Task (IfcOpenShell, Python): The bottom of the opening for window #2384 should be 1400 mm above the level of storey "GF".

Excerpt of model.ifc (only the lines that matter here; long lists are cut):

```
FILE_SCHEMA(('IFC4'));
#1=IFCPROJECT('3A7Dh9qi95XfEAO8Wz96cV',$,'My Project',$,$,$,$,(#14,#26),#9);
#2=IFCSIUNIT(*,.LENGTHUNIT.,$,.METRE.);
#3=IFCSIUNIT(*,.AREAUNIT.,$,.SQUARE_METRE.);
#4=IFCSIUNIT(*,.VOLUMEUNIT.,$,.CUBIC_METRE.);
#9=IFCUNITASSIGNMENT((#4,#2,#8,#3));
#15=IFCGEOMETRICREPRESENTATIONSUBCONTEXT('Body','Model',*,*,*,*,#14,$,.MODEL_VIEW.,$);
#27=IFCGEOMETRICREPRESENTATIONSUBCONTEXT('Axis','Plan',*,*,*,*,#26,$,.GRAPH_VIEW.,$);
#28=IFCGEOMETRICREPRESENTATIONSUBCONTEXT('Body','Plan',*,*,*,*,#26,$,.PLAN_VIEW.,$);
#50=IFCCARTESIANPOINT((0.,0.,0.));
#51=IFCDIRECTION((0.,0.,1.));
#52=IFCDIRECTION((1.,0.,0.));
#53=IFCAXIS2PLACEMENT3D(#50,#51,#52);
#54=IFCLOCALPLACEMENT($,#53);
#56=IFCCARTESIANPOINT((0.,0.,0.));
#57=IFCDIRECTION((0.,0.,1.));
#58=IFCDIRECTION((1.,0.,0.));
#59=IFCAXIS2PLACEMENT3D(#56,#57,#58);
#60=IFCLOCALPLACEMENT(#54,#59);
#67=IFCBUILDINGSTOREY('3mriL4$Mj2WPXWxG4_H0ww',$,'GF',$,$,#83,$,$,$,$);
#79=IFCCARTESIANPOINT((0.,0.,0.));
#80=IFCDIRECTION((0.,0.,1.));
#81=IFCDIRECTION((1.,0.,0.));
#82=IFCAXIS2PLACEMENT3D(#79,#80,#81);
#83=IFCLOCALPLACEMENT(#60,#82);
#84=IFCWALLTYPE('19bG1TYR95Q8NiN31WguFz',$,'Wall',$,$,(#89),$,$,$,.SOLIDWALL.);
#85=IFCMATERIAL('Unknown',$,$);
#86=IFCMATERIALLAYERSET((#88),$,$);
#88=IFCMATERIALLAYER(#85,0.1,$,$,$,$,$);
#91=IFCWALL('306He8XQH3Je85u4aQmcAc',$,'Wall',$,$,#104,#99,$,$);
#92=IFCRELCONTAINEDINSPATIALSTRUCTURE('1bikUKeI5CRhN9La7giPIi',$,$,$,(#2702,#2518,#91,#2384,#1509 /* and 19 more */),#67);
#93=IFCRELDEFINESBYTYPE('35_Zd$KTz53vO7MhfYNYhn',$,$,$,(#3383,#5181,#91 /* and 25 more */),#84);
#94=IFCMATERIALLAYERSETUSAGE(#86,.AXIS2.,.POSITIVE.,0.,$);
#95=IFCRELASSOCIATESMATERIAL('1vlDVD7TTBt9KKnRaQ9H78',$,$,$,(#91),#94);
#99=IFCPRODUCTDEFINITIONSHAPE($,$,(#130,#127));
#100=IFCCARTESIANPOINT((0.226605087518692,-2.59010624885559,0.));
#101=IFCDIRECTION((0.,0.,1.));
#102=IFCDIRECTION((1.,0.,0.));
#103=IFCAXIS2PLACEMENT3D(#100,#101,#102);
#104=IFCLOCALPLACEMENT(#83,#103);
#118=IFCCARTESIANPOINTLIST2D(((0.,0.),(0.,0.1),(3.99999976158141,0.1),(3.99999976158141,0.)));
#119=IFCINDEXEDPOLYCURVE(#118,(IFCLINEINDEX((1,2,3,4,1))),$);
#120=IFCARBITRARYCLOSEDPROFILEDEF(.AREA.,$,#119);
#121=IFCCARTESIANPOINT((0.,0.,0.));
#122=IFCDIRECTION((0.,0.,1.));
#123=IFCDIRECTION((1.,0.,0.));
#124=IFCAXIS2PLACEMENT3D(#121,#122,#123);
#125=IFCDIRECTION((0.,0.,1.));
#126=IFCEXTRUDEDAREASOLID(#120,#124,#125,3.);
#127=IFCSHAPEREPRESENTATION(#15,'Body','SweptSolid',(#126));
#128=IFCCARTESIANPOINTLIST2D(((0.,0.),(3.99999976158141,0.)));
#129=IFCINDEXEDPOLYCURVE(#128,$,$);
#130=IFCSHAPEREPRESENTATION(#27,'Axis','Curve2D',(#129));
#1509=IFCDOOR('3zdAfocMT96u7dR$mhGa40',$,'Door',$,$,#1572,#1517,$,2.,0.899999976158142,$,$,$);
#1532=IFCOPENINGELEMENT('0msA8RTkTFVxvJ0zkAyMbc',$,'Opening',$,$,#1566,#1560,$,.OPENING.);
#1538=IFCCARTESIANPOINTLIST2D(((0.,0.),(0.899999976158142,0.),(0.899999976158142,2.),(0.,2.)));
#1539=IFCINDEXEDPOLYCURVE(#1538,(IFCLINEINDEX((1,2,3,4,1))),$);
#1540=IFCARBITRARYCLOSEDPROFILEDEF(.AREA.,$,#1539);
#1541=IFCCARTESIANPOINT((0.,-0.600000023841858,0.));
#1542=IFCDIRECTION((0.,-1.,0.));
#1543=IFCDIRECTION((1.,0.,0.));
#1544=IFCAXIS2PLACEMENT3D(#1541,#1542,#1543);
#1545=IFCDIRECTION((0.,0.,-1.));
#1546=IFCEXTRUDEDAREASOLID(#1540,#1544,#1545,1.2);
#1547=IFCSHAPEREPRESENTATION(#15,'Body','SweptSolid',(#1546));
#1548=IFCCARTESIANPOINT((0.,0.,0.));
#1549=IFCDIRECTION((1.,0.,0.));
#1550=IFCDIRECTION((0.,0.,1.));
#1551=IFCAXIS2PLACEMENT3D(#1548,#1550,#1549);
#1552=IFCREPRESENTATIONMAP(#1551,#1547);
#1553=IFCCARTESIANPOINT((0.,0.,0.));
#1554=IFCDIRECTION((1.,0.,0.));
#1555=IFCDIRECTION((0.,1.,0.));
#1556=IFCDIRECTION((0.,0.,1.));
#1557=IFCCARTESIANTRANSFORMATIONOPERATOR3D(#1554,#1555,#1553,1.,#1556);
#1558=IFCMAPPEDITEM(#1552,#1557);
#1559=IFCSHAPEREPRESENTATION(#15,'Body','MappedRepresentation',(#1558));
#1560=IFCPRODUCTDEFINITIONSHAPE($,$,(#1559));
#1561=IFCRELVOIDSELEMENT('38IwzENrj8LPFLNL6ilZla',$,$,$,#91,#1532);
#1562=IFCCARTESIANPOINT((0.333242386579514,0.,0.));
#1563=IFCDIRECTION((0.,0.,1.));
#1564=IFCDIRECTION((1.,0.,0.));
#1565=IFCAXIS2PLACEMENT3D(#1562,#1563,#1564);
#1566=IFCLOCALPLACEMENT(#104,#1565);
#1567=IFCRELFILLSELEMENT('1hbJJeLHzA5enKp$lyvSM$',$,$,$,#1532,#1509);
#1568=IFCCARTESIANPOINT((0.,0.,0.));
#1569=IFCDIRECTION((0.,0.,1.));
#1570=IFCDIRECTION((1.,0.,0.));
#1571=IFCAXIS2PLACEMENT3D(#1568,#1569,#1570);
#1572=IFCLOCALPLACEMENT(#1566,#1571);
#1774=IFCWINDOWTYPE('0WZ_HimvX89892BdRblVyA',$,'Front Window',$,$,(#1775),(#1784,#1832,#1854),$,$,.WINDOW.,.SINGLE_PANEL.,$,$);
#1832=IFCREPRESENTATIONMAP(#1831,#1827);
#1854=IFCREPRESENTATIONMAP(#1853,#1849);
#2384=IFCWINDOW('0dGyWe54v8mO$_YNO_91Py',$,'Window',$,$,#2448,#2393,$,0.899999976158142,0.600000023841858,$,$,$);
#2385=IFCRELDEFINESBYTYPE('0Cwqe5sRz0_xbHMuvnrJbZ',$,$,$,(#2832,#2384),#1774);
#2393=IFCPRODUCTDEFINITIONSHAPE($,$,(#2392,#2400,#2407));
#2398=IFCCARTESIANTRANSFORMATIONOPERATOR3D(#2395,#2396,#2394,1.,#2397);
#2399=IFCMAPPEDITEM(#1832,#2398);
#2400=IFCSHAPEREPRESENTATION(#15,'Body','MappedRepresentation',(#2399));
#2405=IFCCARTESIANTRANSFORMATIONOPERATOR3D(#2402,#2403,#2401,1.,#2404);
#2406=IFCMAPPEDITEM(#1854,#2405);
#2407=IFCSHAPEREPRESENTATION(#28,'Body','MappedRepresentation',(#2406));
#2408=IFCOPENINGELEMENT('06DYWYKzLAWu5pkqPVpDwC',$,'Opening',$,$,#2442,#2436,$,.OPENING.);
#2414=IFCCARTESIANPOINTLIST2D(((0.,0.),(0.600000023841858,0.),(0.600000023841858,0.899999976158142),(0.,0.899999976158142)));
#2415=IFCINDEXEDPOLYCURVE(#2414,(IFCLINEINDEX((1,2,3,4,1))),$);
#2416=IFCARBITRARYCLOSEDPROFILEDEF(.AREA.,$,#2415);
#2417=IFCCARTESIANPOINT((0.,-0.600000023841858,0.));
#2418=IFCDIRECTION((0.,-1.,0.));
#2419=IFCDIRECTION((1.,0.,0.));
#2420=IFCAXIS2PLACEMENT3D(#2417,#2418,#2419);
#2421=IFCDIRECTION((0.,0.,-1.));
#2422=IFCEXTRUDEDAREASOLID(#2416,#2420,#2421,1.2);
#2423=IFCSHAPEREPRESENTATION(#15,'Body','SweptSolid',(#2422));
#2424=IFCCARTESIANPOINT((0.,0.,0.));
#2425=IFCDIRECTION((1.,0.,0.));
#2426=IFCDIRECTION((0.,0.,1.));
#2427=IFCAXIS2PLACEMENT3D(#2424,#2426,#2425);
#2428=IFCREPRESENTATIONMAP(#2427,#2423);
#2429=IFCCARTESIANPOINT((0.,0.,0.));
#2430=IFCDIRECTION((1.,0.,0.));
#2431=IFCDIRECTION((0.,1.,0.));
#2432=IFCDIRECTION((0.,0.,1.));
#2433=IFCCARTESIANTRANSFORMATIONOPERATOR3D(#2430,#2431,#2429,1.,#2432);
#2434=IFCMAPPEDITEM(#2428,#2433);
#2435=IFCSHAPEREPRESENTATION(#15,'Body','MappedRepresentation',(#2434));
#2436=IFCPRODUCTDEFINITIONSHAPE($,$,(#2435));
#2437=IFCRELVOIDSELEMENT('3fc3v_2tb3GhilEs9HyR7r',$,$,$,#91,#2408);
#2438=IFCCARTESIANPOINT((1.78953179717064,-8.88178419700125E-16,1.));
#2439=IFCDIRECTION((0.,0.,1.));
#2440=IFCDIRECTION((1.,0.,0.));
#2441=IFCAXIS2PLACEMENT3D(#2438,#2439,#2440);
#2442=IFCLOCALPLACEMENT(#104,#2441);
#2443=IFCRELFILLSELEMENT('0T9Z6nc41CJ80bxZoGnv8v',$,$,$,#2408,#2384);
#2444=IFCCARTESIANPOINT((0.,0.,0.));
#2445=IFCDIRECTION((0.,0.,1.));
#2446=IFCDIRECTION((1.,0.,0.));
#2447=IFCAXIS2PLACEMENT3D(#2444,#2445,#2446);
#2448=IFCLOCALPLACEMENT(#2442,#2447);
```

```python
import numpy as np
import ifcopenshell
import ifcopenshell.api.geometry
import ifcopenshell.geom
import ifcopenshell.util.element
import ifcopenshell.util.placement
import ifcopenshell.util.shape
import ifcopenshell.util.unit

model = ifcopenshell.open("model.ifc")
unit_scale = ifcopenshell.util.unit.calculate_unit_scale(model)

window = model.by_guid("0dGyWe54v8mO$_YNO_91Py")
opening = window.FillsVoids[0].RelatingOpeningElement
storey = ifcopenshell.util.element.get_container(window, ifc_class="IfcBuildingStorey")
level = ifcopenshell.util.placement.get_local_placement(storey.ObjectPlacement)[2, 3]

# The opening's origin need not be at the sill, so measure its lowest point.
shape = ifcopenshell.geom.create_shape(ifcopenshell.geom.settings(), opening)
bottom = ifcopenshell.util.shape.get_shape_bottom_elevation(shape, shape.geometry) / unit_scale
dz = level + 1.4 / unit_scale - bottom

shift = np.array([0.0, 0.0, dz])
# The window is placed relative to its opening, so it follows when the opening moves.
matrix = ifcopenshell.util.placement.get_local_placement(opening.ObjectPlacement)
matrix[:3, 3] += shift
ifcopenshell.api.geometry.edit_object_placement(
    model, product=opening, matrix=matrix, is_si=False, should_transform_children=True
)

print(f"moved by {dz * unit_scale:+.3f} m")

model.write("model_rev.ifc")
```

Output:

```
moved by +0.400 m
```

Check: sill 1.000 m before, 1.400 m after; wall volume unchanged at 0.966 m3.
